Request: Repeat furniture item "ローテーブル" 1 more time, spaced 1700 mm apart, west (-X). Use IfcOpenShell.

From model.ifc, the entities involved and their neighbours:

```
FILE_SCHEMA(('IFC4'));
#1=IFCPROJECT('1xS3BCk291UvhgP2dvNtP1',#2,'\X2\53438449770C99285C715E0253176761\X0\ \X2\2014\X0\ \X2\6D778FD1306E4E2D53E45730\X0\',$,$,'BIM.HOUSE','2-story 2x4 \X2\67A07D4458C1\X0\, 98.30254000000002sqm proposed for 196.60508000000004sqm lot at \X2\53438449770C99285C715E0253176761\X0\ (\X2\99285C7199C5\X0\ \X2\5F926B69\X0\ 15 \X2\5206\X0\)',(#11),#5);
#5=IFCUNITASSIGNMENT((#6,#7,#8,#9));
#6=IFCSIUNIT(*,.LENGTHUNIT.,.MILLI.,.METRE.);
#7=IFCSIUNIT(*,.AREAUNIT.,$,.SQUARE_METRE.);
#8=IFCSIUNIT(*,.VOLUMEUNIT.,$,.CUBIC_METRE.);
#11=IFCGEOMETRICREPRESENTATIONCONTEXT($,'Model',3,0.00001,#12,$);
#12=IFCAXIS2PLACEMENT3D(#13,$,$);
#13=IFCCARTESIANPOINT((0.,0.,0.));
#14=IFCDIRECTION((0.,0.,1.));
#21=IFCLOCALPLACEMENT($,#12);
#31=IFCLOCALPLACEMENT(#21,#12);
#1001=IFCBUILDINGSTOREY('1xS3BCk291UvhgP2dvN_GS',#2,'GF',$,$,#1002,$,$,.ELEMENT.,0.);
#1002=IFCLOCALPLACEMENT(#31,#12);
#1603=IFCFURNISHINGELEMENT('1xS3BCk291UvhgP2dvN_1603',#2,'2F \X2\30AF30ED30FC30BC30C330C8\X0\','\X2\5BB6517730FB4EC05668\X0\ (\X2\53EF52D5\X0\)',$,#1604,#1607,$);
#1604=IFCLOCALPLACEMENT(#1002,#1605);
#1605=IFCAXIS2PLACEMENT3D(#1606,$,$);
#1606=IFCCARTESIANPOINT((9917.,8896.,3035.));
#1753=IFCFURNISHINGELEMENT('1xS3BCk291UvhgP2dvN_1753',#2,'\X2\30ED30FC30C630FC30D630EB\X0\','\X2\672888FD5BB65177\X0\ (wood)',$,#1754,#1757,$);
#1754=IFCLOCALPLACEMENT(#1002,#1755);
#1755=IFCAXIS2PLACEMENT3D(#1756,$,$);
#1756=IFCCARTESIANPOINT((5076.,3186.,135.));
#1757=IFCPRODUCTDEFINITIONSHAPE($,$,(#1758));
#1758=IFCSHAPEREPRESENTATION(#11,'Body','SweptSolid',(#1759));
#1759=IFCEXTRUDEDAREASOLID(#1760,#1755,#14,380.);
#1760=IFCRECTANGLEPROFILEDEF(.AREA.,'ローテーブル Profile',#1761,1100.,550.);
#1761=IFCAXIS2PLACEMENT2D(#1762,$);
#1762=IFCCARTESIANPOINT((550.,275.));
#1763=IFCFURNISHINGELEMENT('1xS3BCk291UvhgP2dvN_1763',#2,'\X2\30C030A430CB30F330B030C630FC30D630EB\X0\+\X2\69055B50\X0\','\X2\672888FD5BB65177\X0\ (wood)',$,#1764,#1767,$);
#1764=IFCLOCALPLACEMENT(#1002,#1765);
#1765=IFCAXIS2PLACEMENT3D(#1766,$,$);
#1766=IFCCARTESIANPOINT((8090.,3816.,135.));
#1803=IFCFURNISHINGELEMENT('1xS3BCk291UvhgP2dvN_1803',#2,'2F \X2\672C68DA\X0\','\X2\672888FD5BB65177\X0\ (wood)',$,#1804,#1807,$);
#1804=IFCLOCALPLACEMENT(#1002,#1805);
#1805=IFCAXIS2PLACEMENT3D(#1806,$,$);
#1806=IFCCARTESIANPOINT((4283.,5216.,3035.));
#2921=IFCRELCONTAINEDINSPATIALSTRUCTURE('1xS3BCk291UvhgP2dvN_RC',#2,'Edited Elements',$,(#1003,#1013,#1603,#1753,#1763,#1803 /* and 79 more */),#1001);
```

```python
import numpy as np
import ifcopenshell
import ifcopenshell.api.geometry
import ifcopenshell.api.root
import ifcopenshell.util.element
import ifcopenshell.util.placement
import ifcopenshell.util.unit

model = ifcopenshell.open("model.ifc")
unit_scale = ifcopenshell.util.unit.calculate_unit_scale(model)


def reuse_history(source, copy):
    """copy_class also copies each property set's owner history, people and application; keep the originals."""
    for rel in copy.IsDefinedBy:
        if rel.is_a("IfcRelDefinesByProperties") and (history := rel.RelatingPropertyDefinition.OwnerHistory):
            rel.RelatingPropertyDefinition.OwnerHistory = source.OwnerHistory
            ifcopenshell.util.element.remove_deep2(model, history)


source = model.by_id(1753)
base = ifcopenshell.util.placement.get_local_placement(source.ObjectPlacement)
step = np.array([-1.0, 0.0, 0.0]) * 1.7 / unit_scale

for i in range(1, 2):
    copy = ifcopenshell.api.root.copy_class(model, product=source)
    copy.Representation = ifcopenshell.util.element.copy_deep(
        model, source.Representation, exclude=["IfcGeometricRepresentationContext", "IfcRepresentationMap"]
    )
    reuse_history(source, copy)
    matrix = base.copy()
    matrix[:3, 3] += i * step
    print("added at", matrix[:3, 3].round(3) + 0.0)
    ifcopenshell.api.geometry.edit_object_placement(model, product=copy, matrix=matrix, is_si=False)

model.write("model_v2.ifc")
```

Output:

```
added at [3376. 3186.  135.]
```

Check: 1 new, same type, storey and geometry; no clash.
